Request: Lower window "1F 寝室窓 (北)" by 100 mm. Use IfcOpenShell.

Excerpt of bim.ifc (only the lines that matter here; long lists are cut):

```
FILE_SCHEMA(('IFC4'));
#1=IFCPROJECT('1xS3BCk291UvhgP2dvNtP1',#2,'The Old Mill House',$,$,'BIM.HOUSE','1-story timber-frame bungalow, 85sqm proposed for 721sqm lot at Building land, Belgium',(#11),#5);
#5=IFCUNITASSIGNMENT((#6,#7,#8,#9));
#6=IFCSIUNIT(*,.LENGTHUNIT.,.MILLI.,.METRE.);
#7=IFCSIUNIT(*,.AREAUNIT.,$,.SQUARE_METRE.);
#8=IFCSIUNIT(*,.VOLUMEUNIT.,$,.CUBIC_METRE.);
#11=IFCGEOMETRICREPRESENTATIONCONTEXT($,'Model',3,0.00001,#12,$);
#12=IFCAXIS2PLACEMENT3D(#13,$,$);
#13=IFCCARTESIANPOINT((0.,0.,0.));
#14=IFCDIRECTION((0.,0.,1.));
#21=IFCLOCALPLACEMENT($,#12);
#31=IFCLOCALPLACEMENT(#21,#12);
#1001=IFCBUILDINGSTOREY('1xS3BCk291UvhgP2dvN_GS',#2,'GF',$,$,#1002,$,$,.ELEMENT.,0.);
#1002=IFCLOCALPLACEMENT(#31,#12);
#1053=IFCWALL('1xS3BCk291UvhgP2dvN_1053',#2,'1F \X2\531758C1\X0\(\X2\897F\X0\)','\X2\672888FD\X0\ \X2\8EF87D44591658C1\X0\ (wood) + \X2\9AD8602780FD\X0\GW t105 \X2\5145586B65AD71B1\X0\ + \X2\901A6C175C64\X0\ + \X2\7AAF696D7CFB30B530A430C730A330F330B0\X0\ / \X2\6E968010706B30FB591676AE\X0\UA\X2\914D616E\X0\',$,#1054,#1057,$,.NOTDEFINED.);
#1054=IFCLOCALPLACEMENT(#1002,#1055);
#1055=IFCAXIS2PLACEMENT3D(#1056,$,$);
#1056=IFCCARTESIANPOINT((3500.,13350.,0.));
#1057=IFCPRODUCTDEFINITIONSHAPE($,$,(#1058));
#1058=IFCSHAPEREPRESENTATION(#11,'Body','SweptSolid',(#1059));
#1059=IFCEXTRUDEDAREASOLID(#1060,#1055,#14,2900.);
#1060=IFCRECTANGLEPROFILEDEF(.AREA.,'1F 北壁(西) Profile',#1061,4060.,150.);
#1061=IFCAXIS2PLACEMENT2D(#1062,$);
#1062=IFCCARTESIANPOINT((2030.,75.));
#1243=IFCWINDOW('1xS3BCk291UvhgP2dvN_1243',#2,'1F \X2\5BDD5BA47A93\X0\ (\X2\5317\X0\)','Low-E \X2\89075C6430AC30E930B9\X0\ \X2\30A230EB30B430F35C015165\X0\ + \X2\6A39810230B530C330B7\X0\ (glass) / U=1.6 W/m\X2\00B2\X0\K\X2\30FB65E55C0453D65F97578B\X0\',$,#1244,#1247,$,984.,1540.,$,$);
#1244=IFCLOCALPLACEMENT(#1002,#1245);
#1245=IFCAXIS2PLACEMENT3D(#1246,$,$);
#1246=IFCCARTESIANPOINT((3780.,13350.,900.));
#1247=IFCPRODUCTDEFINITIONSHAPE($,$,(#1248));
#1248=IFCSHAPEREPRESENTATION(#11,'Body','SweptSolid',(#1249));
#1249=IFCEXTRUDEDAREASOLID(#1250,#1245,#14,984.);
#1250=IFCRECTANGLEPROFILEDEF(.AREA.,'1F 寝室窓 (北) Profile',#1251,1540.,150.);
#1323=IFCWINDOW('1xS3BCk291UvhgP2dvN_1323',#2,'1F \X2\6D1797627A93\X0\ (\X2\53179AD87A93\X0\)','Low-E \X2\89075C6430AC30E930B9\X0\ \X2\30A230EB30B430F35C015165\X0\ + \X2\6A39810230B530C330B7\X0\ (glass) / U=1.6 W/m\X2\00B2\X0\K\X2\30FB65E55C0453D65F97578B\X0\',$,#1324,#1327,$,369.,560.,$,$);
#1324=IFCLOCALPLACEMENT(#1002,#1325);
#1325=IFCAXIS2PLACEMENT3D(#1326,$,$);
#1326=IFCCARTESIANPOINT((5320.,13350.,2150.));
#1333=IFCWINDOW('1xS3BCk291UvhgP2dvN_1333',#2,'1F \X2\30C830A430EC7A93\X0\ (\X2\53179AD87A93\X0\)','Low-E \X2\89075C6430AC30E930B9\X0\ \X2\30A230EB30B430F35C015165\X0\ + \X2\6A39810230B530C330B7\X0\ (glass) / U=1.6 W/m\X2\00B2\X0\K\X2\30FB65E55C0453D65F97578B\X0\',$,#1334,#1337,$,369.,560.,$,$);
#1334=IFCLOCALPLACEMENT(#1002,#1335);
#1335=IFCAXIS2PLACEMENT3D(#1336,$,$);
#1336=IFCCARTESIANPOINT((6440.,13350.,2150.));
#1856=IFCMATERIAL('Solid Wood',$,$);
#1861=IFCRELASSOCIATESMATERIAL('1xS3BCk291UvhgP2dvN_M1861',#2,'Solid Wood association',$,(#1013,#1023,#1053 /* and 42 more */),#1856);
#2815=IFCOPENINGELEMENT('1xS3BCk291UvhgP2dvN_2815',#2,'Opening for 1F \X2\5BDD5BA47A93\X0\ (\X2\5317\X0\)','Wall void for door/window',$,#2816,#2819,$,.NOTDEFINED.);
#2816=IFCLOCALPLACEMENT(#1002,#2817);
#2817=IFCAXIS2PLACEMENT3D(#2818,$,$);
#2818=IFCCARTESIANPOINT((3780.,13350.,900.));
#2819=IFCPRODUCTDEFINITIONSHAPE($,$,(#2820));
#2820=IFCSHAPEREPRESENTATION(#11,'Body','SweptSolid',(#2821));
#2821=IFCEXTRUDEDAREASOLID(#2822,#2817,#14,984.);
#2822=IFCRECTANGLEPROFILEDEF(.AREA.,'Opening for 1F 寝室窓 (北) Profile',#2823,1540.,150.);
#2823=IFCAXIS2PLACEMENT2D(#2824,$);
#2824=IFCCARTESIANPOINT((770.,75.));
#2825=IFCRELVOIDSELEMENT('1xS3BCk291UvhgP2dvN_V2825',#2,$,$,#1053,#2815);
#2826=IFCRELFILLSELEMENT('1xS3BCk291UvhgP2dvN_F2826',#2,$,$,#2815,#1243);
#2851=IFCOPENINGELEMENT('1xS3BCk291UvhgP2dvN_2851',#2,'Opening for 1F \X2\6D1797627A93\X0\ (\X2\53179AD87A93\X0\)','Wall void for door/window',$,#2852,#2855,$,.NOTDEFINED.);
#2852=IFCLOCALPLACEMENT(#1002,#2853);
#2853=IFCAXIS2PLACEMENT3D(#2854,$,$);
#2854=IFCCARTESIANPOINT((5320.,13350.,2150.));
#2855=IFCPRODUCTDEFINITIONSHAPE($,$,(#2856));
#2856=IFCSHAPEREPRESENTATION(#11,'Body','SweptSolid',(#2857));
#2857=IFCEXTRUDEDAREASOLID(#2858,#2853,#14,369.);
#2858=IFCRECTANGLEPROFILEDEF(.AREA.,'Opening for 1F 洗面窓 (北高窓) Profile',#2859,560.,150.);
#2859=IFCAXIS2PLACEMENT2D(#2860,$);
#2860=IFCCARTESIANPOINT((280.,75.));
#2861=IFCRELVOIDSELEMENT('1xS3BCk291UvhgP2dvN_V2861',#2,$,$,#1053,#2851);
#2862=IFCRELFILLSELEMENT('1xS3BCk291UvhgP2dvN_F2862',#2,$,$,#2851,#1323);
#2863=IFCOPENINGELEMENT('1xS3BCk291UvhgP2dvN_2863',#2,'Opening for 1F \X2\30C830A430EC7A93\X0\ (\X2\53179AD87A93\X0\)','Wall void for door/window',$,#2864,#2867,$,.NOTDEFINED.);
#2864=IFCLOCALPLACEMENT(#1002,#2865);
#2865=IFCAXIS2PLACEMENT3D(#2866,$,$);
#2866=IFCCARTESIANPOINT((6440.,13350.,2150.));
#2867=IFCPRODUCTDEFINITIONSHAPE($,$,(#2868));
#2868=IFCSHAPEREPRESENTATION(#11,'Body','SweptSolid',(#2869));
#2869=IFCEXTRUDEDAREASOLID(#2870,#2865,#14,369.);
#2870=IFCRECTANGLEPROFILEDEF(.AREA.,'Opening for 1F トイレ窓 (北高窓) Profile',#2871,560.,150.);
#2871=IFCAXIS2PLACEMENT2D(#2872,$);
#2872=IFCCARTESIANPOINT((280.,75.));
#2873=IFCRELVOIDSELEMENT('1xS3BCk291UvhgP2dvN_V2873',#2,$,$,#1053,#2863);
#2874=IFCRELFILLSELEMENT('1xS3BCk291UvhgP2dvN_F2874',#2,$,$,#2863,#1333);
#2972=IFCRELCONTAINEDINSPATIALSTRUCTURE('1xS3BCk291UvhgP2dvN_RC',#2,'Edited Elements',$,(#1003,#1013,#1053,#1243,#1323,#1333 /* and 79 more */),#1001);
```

```python
import numpy as np
import ifcopenshell
import ifcopenshell.api.geometry
import ifcopenshell.util.placement
import ifcopenshell.util.unit

model = ifcopenshell.open("bim.ifc")
unit_scale = ifcopenshell.util.unit.calculate_unit_scale(model)

window = model.by_guid("1xS3BCk291UvhgP2dvN_1243")
opening = window.FillsVoids[0].RelatingOpeningElement
dz = -0.1 / unit_scale

shift = np.array([0.0, 0.0, dz])
# The window is not placed relative to its opening, so move both.
for product in (opening, window):
    matrix = ifcopenshell.util.placement.get_local_placement(product.ObjectPlacement)
    matrix[:3, 3] += shift
    ifcopenshell.api.geometry.edit_object_placement(model, product=product, matrix=matrix, is_si=False)

print(f"moved by {dz * unit_scale:+.3f} m")

model.write("bim-out.ifc")
```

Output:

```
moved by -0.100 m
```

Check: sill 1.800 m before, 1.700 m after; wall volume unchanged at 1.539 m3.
